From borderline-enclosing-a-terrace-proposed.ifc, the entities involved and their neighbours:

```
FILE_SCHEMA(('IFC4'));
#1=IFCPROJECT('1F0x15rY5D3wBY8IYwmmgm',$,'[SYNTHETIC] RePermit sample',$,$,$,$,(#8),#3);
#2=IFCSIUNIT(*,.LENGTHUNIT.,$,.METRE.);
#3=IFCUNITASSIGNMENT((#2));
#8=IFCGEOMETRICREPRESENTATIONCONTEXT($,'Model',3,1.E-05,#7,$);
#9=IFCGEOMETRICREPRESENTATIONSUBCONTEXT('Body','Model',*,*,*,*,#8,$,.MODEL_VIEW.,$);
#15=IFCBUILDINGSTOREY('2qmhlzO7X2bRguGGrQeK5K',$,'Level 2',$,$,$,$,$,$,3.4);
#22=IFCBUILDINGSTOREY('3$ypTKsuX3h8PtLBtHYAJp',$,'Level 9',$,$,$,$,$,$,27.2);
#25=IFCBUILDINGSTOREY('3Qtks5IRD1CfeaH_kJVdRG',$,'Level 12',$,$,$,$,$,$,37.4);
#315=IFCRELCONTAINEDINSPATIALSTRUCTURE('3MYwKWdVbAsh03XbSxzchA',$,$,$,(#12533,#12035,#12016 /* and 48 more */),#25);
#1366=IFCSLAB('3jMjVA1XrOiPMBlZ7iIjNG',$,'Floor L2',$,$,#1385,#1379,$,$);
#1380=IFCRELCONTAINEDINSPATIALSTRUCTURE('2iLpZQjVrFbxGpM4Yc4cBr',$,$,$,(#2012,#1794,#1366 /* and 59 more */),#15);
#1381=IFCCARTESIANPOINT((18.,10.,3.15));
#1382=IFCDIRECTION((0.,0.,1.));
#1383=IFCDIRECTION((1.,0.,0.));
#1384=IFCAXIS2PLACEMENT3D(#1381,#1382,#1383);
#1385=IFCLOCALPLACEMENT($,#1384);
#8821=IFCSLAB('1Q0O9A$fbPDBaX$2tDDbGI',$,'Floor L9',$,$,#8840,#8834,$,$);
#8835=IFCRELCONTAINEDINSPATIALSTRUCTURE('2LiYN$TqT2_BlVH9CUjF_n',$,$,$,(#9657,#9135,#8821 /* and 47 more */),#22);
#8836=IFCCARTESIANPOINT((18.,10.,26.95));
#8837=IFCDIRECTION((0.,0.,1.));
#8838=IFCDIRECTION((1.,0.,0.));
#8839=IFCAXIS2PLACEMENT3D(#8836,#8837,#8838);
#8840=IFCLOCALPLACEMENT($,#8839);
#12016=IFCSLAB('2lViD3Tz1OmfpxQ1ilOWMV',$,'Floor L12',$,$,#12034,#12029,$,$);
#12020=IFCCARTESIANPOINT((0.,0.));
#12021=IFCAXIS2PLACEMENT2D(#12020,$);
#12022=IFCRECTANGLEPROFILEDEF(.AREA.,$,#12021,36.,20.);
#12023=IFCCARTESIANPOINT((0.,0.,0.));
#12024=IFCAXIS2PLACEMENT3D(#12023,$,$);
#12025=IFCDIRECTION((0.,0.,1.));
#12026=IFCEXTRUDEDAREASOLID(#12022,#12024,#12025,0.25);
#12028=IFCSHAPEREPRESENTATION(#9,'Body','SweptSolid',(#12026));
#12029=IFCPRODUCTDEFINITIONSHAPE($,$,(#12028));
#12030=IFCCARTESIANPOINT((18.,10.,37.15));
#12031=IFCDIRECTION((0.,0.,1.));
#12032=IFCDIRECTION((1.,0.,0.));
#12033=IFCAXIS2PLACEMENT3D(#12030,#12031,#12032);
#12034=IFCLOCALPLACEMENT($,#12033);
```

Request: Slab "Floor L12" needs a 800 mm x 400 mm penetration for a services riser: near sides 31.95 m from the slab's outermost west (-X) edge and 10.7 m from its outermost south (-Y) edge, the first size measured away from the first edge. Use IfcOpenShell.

```python
import numpy as np
import ifcopenshell
import ifcopenshell.api.feature
import ifcopenshell.api.geometry
import ifcopenshell.api.root
import ifcopenshell.geom
import ifcopenshell.util.placement
import ifcopenshell.util.representation
import ifcopenshell.util.shape
import ifcopenshell.util.unit

model = ifcopenshell.open("borderline-enclosing-a-terrace-proposed.ifc")
unit_scale = ifcopenshell.util.unit.calculate_unit_scale(model)
settings = ifcopenshell.geom.settings()


def volume(element):
    """Net volume in cubic metres, openings subtracted."""
    shape = ifcopenshell.geom.create_shape(settings, element)
    return ifcopenshell.util.shape.get_volume(shape.geometry)


slab = model.by_guid("2lViD3Tz1OmfpxQ1ilOWMV")
before = volume(slab)

# Extent in the slab's own axes, in metres. The edges named are its -X and -Y sides.
slab_shape = ifcopenshell.geom.create_shape(settings, slab)
vertices = ifcopenshell.util.shape.get_vertices(slab_shape.geometry)
x_min, y_min, bottom = vertices.min(axis=0)
top = vertices[:, 2].max()

opening = ifcopenshell.api.root.create_entity(model, ifc_class="IfcOpeningElement", name="Services riser opening", predefined_type="OPENING")
context = ifcopenshell.util.representation.get_context(model, "Model", "Body", "MODEL_VIEW")
width, depth = 0.8, 0.4
outline = [(0.0, 0.0), (width, 0.0), (width, depth), (0.0, depth), (0.0, 0.0)]
# Overshoot both faces by 50 mm so the cut is clean.
shape = ifcopenshell.api.geometry.add_slab_representation(
    model, context=context, depth=top - bottom + 0.1, polyline=outline
)
ifcopenshell.api.geometry.assign_representation(model, product=opening, representation=shape)

matrix = ifcopenshell.util.placement.get_local_placement(slab.ObjectPlacement)
matrix[:, 3] = matrix @ np.append(np.array([x_min + 31.95, y_min + 10.7, bottom - 0.05]) / unit_scale, 1.0)
ifcopenshell.api.geometry.edit_object_placement(model, product=opening, matrix=matrix, is_si=False)
ifcopenshell.api.feature.add_feature(model, feature=opening, element=slab)

after = volume(slab)

print(f"slab volume {before:.3f} -> {after:.3f} m3")

model.write("borderline-enclosing-a-terrace-proposed_updated.ifc")
```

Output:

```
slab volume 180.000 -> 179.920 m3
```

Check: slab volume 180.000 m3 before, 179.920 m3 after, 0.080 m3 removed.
